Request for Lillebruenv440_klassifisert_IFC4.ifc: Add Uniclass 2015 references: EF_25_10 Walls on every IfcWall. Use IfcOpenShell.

First a look at what the model holds.

```python
import ifcopenshell

model = ifcopenshell.open("Lillebruenv440_klassifisert_IFC4.ifc")
print(model.schema)
print("classifications:", [c.Name for c in model.by_type("IfcClassification")])
for ifc_class in ("IfcDoor", "IfcRoof", "IfcStair", "IfcWall", "IfcWindow"):
    print(ifc_class, len(model.by_type(ifc_class)))
```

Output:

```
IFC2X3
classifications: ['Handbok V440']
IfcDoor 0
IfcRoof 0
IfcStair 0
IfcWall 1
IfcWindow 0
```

```python
import ifcopenshell
import ifcopenshell.api.classification

model = ifcopenshell.open("Lillebruenv440_klassifisert_IFC4.ifc")

# IFC2X3 requires Source and Edition and has no link from the project to the system.
system = model.create_entity("IfcClassification", Source="NBS", Edition="2015", Name="Uniclass 2015")

codes = {
    "IfcWall": ("EF_25_10", "Walls"),
}
for ifc_class, (code, name) in codes.items():
    products = model.by_type(ifc_class)
    ifcopenshell.api.classification.add_reference(
        model, products=products, classification=system, identification=code, name=name
    )
    print(code, len(products))

model.write("Lillebruenv440_klassifisert_IFC4_edited.ifc")
```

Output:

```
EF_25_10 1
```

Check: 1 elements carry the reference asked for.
